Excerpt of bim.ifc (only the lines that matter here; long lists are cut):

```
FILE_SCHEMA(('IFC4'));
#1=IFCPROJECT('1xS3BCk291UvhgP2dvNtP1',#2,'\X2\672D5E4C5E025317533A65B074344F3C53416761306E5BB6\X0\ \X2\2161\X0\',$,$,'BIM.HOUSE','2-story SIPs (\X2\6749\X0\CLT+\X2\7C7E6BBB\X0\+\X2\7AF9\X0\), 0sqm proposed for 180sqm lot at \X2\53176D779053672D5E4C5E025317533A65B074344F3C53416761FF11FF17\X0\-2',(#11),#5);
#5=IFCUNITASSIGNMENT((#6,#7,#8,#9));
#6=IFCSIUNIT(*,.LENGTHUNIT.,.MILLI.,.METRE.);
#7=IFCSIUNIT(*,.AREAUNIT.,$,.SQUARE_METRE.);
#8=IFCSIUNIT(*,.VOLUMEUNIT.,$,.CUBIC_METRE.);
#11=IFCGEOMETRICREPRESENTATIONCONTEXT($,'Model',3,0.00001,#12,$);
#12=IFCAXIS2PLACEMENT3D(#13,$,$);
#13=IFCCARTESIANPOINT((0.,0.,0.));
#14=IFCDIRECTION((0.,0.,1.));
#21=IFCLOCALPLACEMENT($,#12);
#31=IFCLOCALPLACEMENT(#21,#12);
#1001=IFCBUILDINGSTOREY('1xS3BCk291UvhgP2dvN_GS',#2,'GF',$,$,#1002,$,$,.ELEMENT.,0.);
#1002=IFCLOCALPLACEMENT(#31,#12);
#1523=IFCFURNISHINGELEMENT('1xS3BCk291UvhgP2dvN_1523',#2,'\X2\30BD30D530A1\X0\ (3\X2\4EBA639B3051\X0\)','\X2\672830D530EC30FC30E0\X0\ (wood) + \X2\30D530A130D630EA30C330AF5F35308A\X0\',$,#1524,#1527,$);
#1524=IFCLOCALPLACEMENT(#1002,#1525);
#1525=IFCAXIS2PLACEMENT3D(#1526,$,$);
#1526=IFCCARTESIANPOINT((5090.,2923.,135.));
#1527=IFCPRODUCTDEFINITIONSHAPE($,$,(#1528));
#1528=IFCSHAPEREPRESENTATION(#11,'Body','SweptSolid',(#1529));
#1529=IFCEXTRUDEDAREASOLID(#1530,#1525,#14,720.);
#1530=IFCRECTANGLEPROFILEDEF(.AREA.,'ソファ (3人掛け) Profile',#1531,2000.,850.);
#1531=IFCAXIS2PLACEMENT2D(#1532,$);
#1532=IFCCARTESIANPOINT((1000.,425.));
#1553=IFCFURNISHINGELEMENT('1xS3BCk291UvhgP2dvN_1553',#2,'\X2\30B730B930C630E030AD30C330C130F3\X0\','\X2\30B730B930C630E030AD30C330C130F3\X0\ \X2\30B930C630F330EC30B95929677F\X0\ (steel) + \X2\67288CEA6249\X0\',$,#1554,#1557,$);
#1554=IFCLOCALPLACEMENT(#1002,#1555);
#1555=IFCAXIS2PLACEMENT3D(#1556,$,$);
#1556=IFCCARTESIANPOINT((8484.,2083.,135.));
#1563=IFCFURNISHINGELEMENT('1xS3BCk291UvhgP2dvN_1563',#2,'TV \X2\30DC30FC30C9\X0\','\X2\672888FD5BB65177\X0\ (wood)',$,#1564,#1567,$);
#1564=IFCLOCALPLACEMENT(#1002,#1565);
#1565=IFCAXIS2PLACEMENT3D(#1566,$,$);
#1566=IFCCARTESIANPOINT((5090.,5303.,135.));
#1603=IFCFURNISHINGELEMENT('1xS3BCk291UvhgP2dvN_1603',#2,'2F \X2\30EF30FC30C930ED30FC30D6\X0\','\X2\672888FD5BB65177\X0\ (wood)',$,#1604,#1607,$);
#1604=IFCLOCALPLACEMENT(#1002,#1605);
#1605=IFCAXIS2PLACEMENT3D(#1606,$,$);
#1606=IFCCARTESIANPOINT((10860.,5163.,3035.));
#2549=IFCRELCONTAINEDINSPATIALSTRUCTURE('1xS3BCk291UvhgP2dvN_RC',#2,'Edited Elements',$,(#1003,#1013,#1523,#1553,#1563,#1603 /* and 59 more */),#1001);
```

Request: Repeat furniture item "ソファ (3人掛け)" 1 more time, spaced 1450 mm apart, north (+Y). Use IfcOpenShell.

```python
import numpy as np
import ifcopenshell
import ifcopenshell.api.geometry
import ifcopenshell.api.root
import ifcopenshell.util.element
import ifcopenshell.util.placement
import ifcopenshell.util.unit

model = ifcopenshell.open("bim.ifc")
unit_scale = ifcopenshell.util.unit.calculate_unit_scale(model)


def reuse_history(source, copy):
    """copy_class also copies each property set's owner history, people and application; keep the originals."""
    for rel in copy.IsDefinedBy:
        if rel.is_a("IfcRelDefinesByProperties") and (history := rel.RelatingPropertyDefinition.OwnerHistory):
            rel.RelatingPropertyDefinition.OwnerHistory = source.OwnerHistory
            ifcopenshell.util.element.remove_deep2(model, history)


source = model.by_guid("1xS3BCk291UvhgP2dvN_1523")
base = ifcopenshell.util.placement.get_local_placement(source.ObjectPlacement)
step = np.array([0.0, 1.0, 0.0]) * 1.45 / unit_scale

for i in range(1, 2):
    copy = ifcopenshell.api.root.copy_class(model, product=source)
    copy.Representation = ifcopenshell.util.element.copy_deep(
        model, source.Representation, exclude=["IfcGeometricRepresentationContext", "IfcRepresentationMap"]
    )
    reuse_history(source, copy)
    matrix = base.copy()
    matrix[:3, 3] += i * step
    print("added at", matrix[:3, 3].round(3) + 0.0)
    ifcopenshell.api.geometry.edit_object_placement(model, product=copy, matrix=matrix, is_si=False)

model.write("bim_edited.ifc")
```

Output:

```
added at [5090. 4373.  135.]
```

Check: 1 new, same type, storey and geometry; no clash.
